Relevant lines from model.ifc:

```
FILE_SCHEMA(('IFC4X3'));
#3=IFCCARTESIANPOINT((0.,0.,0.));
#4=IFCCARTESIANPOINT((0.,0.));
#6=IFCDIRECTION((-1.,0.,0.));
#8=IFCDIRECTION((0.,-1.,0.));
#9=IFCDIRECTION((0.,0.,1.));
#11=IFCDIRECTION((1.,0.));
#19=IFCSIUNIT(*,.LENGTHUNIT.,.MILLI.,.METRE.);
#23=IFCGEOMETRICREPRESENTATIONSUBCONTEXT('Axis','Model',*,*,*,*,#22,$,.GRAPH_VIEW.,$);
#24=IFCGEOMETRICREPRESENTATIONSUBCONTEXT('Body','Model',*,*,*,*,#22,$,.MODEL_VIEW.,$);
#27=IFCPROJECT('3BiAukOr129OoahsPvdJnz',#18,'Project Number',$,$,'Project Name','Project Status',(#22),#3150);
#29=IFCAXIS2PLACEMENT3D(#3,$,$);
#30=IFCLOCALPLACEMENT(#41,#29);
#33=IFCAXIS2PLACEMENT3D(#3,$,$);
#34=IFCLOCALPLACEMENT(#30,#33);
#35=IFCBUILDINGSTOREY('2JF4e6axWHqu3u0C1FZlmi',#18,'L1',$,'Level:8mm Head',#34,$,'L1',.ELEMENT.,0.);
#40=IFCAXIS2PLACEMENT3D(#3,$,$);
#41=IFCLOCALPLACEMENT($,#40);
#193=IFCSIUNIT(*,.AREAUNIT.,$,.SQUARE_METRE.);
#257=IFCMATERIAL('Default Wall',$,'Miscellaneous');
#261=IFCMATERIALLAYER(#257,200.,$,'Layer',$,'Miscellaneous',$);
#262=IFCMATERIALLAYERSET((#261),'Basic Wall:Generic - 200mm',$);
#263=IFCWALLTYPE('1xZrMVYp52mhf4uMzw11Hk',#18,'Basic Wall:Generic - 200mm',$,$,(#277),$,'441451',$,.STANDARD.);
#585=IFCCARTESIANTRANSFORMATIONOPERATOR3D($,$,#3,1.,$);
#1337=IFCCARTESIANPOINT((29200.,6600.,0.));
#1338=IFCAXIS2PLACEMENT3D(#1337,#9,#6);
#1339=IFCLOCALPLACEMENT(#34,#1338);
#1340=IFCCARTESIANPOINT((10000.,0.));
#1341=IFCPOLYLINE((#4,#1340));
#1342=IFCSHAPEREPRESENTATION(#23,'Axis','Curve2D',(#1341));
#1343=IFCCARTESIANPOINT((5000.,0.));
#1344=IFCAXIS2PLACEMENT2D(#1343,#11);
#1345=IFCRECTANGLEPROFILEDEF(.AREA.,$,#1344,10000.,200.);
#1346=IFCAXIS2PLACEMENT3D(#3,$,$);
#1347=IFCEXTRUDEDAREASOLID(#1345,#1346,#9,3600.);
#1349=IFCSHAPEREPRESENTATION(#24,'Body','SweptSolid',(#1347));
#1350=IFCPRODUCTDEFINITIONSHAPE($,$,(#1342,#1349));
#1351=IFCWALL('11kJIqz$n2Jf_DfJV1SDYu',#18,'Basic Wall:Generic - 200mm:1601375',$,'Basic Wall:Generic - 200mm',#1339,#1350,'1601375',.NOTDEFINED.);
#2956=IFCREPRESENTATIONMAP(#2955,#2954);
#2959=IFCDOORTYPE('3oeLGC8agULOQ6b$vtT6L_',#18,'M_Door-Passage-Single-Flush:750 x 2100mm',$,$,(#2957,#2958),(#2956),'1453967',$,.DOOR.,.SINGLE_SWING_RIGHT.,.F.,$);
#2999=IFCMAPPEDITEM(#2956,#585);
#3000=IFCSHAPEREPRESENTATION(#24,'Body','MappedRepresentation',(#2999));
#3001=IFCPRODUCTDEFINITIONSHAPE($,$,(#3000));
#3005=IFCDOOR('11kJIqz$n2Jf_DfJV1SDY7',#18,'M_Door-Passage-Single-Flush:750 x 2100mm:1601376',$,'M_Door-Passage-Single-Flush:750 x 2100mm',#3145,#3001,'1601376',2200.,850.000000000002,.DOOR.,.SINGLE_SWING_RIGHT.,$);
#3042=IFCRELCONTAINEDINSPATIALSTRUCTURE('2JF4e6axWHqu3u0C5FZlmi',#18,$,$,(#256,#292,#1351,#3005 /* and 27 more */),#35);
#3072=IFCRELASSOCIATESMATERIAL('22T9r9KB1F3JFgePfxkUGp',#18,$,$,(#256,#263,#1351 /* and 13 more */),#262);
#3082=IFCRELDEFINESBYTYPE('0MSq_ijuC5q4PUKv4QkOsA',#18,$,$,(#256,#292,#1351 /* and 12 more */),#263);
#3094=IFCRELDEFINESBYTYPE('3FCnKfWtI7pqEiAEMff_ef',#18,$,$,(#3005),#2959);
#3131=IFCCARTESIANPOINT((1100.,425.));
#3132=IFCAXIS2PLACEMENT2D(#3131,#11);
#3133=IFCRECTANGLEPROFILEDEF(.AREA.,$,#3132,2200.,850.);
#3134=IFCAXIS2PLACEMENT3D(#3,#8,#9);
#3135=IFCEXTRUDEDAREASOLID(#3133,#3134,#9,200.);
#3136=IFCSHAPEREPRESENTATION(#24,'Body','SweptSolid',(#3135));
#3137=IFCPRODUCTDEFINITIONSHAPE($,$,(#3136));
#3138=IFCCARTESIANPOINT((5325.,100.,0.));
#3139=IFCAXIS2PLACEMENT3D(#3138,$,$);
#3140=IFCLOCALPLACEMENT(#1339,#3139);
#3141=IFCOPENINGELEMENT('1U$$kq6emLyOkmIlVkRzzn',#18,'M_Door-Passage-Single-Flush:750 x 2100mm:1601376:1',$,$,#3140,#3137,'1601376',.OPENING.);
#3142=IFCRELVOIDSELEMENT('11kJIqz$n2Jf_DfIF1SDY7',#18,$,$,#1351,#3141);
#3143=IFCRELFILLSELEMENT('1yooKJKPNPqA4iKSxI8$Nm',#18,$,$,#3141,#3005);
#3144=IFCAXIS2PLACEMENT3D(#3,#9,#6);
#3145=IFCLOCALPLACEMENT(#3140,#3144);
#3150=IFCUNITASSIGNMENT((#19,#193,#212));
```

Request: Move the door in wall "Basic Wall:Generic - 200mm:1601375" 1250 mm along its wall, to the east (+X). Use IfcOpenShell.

```python
import ifcopenshell
import ifcopenshell.api.geometry
import ifcopenshell.util.placement
import ifcopenshell.util.unit

model = ifcopenshell.open("model.ifc")
unit_scale = ifcopenshell.util.unit.calculate_unit_scale(model)

door = model.by_guid("11kJIqz$n2Jf_DfJV1SDY7")
opening = door.FillsVoids[0].RelatingOpeningElement
wall = opening.VoidsElements[0].RelatingBuildingElement

wall_matrix = ifcopenshell.util.placement.get_local_placement(wall.ObjectPlacement)
shift = wall_matrix[:3, 0] * -1.25 / unit_scale
before = ifcopenshell.util.placement.get_local_placement(door.ObjectPlacement)[:3, 3].copy()

# The door is placed relative to its opening, so it follows when the opening moves.
matrix = ifcopenshell.util.placement.get_local_placement(opening.ObjectPlacement)
matrix[:3, 3] += shift
ifcopenshell.api.geometry.edit_object_placement(
    model, product=opening, matrix=matrix, is_si=False, should_transform_children=True
)

after = ifcopenshell.util.placement.get_local_placement(door.ObjectPlacement)[:3, 3]
print("door moved by", (after - before).round(3) + 0.0)

model.write("model_rev.ifc")
```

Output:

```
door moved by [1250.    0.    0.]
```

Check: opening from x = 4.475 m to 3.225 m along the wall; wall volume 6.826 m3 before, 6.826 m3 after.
